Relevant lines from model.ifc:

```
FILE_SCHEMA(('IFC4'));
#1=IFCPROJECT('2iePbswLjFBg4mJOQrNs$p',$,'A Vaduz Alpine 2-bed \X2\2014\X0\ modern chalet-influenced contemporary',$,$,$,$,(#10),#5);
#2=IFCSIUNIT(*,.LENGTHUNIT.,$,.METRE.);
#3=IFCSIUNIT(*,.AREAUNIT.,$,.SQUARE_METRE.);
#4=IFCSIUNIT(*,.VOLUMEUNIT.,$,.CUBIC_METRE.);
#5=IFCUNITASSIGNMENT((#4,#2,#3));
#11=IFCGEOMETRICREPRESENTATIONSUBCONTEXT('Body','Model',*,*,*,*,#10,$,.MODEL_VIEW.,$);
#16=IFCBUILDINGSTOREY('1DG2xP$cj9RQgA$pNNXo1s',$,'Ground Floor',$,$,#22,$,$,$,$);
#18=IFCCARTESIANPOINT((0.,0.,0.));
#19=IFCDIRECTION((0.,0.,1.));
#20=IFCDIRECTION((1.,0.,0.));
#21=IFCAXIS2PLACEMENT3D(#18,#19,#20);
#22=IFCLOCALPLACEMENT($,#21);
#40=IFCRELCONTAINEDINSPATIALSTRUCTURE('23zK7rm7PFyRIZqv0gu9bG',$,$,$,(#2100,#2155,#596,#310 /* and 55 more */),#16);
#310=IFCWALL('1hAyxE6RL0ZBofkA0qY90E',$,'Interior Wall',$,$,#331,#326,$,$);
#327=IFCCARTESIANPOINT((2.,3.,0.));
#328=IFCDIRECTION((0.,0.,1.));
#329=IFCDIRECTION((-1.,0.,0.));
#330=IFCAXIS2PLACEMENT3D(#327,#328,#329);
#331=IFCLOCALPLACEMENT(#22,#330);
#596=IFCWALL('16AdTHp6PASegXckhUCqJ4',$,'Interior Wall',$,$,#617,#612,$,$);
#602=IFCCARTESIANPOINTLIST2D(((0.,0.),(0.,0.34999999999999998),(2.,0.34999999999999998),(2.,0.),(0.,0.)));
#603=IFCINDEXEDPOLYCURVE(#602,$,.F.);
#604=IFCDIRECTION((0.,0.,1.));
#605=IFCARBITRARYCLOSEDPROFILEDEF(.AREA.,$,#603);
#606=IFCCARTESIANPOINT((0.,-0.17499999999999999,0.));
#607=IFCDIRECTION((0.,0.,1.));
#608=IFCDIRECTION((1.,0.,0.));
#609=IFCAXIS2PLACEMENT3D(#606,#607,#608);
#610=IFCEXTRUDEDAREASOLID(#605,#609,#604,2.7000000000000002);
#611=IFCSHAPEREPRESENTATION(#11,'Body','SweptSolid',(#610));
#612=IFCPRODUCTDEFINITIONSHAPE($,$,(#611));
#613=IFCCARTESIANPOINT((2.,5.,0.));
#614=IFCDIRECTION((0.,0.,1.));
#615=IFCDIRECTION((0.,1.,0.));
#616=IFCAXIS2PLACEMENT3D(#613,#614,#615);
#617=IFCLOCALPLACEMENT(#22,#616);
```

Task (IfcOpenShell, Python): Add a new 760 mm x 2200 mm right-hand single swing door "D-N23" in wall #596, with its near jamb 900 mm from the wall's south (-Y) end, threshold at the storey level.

```python
import numpy as np
import ifcopenshell
import ifcopenshell.api.feature
import ifcopenshell.api.geometry
import ifcopenshell.api.root
import ifcopenshell.api.spatial
import ifcopenshell.geom
import ifcopenshell.util.element
import ifcopenshell.util.placement
import ifcopenshell.util.representation
import ifcopenshell.util.shape
import ifcopenshell.util.unit

model = ifcopenshell.open("model.ifc")
unit_scale = ifcopenshell.util.unit.calculate_unit_scale(model)
settings = ifcopenshell.geom.settings()


def volume(element):
    """Net volume in cubic metres, openings subtracted."""
    shape = ifcopenshell.geom.create_shape(settings, element)
    return ifcopenshell.util.shape.get_volume(shape.geometry)


wall = model.by_guid("16AdTHp6PASegXckhUCqJ4")
storey = ifcopenshell.util.element.get_container(wall, ifc_class="IfcBuildingStorey")
context = ifcopenshell.util.representation.get_context(model, "Model", "Body", "MODEL_VIEW")
before = volume(wall)

width, height, from_end, sill = 0.76, 2.2, 0.9, 0.0  # metres

# The wall runs along its own X axis, and the end named is its -X end.
wall_shape = ifcopenshell.geom.create_shape(settings, wall)
x, y, z = ifcopenshell.util.shape.get_vertices(wall_shape.geometry).T
start = x.min() + from_end
face, thickness = float(y.min()), float(y.max() - y.min())
wall_matrix = ifcopenshell.util.placement.get_local_placement(wall.ObjectPlacement)
level = ifcopenshell.util.placement.get_local_placement(storey.ObjectPlacement)[2, 3]


def in_wall(x, y):
    """Placement at x, y metres in the wall's axes, at sill height."""
    matrix = wall_matrix.copy()
    matrix[:, 3] = wall_matrix @ np.array([x / unit_scale, y / unit_scale, 0.0, 1.0])
    matrix[2, 3] = level + sill / unit_scale
    return matrix


# Opening: a box that overshoots both wall faces by 50 mm.
opening = ifcopenshell.api.root.create_entity(model, ifc_class="IfcOpeningElement", predefined_type="OPENING")
box = ifcopenshell.api.geometry.add_wall_representation(
    model, context=context, length=width, height=height, thickness=thickness + 0.1
)
ifcopenshell.api.geometry.assign_representation(model, product=opening, representation=box)
ifcopenshell.api.geometry.edit_object_placement(model, product=opening, matrix=in_wall(start, face - 0.05), is_si=False)
ifcopenshell.api.feature.add_feature(model, feature=opening, element=wall)

door = ifcopenshell.api.root.create_entity(model, ifc_class="IfcDoor", name="D-N23", predefined_type="DOOR")
door.OverallWidth, door.OverallHeight = width / unit_scale, height / unit_scale
door.OperationType = "SINGLE_SWING_RIGHT"
body = ifcopenshell.api.geometry.add_door_representation(
    model,
    context=context,
    overall_width=door.OverallWidth,
    overall_height=door.OverallHeight,
    operation_type="SINGLE_SWING_RIGHT",
    lining_properties={"LiningDepth": thickness / unit_scale, "ThresholdDepth": thickness / unit_scale},
)
ifcopenshell.api.geometry.assign_representation(model, product=door, representation=body)
ifcopenshell.api.spatial.assign_container(model, products=[door], relating_structure=storey)
ifcopenshell.api.feature.add_filling(model, opening=opening, element=door)

# The lining spans the wall, so the door starts at the wall face.
ifcopenshell.api.geometry.edit_object_placement(model, product=door, matrix=in_wall(start, face), is_si=False)

after = volume(wall)

print(f"wall volume {before:.3f} -> {after:.3f} m3")

model.write("model_v2.ifc")
```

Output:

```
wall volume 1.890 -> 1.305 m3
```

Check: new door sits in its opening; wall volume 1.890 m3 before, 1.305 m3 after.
